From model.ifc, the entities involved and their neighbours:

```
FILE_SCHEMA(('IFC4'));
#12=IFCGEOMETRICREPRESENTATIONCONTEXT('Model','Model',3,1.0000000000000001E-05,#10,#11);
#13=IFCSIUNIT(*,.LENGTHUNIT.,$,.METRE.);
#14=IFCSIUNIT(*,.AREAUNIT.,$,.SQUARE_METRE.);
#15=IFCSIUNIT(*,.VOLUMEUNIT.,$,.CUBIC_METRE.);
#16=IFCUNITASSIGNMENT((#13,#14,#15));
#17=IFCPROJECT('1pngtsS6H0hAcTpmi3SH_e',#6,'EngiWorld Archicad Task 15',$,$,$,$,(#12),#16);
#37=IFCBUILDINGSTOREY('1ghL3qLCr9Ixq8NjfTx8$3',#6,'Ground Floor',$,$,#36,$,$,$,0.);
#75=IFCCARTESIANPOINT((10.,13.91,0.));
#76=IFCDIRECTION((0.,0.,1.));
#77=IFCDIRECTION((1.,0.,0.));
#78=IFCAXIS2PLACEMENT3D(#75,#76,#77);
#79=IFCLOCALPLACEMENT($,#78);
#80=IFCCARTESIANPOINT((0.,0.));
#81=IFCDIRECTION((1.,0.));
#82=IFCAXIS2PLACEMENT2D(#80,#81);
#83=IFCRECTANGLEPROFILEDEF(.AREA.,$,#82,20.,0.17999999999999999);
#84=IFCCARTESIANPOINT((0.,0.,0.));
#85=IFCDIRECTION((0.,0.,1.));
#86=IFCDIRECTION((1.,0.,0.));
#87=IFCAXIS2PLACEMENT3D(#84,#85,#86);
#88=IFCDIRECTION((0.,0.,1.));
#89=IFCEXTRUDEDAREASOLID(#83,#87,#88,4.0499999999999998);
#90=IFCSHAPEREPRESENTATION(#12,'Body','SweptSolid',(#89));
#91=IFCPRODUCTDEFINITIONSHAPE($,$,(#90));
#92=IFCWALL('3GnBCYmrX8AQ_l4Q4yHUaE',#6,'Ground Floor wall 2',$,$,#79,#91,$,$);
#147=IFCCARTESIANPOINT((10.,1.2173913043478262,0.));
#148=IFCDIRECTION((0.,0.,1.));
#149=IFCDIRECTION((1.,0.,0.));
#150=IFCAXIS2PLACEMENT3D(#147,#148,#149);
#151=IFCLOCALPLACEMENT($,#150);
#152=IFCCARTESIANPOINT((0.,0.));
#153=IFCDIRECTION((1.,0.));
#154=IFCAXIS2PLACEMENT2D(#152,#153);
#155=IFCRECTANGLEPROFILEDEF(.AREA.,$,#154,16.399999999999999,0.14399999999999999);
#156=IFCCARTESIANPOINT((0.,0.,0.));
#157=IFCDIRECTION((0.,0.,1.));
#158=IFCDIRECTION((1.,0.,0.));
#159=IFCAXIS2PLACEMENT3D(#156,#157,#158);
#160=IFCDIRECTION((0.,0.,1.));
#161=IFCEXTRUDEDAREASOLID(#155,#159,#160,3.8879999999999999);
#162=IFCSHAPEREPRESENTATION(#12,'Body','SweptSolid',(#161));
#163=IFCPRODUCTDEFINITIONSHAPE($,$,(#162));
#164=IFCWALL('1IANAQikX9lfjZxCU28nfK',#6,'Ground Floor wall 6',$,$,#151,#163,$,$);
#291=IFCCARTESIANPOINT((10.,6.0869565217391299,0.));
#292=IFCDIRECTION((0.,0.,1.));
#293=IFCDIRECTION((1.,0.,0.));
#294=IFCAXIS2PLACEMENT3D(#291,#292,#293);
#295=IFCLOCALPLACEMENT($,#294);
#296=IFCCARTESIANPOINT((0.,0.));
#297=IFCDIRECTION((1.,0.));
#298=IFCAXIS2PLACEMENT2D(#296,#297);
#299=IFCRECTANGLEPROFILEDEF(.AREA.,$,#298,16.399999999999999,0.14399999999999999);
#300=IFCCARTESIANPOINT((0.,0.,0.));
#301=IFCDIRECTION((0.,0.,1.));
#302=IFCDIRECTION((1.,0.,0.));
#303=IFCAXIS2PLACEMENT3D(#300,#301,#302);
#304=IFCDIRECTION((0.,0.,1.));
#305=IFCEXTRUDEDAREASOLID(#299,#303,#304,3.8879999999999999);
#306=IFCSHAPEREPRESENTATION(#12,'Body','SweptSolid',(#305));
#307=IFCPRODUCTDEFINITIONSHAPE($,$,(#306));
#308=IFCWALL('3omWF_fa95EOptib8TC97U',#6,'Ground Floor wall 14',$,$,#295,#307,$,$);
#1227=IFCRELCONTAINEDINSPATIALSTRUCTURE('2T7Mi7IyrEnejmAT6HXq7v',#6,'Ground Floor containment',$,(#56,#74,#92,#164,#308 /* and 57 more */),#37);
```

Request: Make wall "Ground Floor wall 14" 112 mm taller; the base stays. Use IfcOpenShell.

```python
import ifcopenshell
import ifcopenshell.geom
import ifcopenshell.util.shape

model = ifcopenshell.open("model.ifc")
settings = ifcopenshell.geom.settings()


def volume(element):
    """Net volume in cubic metres, openings subtracted."""
    shape = ifcopenshell.geom.create_shape(settings, element)
    return ifcopenshell.util.shape.get_volume(shape.geometry)


wall = model.by_guid("3omWF_fa95EOptib8TC97U")
before = volume(wall)

body = next(r for r in wall.Representation.Representations if r.RepresentationIdentifier == "Body")
solid = body.Items[0]
old_height = solid.Depth
solid.Depth += 0.112
after = volume(wall)

print(f"height {old_height:g} -> {solid.Depth:g}, volume {before:.3f} -> {after:.3f} m3")

model.write("model_edited.ifc")
```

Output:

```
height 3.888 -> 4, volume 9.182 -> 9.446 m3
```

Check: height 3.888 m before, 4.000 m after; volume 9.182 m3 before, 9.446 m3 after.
